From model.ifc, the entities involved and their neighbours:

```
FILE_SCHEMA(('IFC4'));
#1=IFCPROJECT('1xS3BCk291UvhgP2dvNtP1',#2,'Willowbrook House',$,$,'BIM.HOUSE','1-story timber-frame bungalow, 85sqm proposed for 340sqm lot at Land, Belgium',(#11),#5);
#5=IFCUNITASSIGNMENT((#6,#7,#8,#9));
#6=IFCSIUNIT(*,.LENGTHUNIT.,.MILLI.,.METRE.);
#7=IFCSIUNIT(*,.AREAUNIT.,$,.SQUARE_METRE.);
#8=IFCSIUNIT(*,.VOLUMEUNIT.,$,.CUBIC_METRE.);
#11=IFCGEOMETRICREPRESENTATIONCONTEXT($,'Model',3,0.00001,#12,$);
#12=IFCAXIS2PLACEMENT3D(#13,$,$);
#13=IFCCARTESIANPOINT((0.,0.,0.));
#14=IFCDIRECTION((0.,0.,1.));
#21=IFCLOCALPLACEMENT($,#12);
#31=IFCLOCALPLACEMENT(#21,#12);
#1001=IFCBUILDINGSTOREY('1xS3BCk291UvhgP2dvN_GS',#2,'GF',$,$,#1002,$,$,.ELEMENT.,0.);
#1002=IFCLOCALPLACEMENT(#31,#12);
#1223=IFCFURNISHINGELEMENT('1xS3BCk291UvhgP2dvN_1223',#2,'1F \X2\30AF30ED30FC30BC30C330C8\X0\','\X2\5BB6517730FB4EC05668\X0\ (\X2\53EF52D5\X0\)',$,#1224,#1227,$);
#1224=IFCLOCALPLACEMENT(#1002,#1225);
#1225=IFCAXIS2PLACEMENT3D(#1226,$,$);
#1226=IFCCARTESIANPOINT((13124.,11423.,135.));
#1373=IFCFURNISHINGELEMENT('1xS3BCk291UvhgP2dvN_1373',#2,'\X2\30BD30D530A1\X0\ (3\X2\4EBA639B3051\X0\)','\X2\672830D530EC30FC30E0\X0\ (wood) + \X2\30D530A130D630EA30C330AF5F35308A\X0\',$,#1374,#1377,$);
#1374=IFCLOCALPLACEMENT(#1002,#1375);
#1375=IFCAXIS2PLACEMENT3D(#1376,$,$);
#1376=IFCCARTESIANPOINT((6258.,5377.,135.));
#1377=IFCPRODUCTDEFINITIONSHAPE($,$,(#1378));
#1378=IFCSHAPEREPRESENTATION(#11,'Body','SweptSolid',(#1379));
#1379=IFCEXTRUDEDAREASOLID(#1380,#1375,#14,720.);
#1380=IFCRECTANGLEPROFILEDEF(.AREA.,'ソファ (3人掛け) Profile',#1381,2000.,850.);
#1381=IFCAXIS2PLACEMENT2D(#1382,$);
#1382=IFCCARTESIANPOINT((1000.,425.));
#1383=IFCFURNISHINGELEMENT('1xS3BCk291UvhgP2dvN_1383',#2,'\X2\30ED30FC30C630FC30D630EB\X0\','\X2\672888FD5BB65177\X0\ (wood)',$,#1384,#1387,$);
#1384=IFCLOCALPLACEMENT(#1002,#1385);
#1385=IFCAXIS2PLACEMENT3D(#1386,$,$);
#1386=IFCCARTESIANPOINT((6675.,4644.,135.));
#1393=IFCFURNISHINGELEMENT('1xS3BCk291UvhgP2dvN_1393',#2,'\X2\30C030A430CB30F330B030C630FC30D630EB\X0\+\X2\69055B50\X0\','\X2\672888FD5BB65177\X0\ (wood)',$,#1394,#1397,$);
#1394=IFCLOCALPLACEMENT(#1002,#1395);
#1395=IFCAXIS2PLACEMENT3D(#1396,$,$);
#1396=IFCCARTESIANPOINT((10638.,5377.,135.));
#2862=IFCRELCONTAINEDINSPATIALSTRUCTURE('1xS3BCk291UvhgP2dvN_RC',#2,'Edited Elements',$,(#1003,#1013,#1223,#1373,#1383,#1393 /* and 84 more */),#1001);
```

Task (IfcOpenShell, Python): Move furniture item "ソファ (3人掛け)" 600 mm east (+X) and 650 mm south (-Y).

```python
import ifcopenshell
import ifcopenshell.api.geometry
import ifcopenshell.util.placement

model = ifcopenshell.open("model.ifc")

item = model.by_guid("1xS3BCk291UvhgP2dvN_1373")
matrix = ifcopenshell.util.placement.get_local_placement(item.ObjectPlacement)
matrix[0, 3] += 600.0
matrix[1, 3] -= 650.0
ifcopenshell.api.geometry.edit_object_placement(model, product=item, matrix=matrix, is_si=False)

print(ifcopenshell.util.placement.get_local_placement(item.ObjectPlacement).round(3) + 0.0)

model.write("model_rev.ifc")
```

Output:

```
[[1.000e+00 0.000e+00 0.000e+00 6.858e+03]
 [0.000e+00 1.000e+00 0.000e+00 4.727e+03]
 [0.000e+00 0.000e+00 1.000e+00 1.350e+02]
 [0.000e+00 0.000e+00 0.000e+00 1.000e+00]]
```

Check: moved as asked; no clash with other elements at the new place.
